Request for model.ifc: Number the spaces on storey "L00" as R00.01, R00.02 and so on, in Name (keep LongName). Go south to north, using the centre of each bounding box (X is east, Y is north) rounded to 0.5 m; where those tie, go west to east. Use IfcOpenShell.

First a look at what the model holds.

```python
import ifcopenshell
import ifcopenshell.util.element
import ifcopenshell.util.placement

model = ifcopenshell.open("model.ifc")
print(model.schema)
storey = next(s for s in model.by_type("IfcBuildingStorey") if s.Name == "L00")
spaces = [e for e in ifcopenshell.util.element.get_decomposition(storey) if e.is_a("IfcSpace")]
for e in sorted(spaces, key=lambda e: e.id()):
    origin = ifcopenshell.util.placement.get_local_placement(e.ObjectPlacement)[:3, 3]
    print(e.id(), e.Name, e.LongName, origin.round(2) + 0.0, sep=" | ")
```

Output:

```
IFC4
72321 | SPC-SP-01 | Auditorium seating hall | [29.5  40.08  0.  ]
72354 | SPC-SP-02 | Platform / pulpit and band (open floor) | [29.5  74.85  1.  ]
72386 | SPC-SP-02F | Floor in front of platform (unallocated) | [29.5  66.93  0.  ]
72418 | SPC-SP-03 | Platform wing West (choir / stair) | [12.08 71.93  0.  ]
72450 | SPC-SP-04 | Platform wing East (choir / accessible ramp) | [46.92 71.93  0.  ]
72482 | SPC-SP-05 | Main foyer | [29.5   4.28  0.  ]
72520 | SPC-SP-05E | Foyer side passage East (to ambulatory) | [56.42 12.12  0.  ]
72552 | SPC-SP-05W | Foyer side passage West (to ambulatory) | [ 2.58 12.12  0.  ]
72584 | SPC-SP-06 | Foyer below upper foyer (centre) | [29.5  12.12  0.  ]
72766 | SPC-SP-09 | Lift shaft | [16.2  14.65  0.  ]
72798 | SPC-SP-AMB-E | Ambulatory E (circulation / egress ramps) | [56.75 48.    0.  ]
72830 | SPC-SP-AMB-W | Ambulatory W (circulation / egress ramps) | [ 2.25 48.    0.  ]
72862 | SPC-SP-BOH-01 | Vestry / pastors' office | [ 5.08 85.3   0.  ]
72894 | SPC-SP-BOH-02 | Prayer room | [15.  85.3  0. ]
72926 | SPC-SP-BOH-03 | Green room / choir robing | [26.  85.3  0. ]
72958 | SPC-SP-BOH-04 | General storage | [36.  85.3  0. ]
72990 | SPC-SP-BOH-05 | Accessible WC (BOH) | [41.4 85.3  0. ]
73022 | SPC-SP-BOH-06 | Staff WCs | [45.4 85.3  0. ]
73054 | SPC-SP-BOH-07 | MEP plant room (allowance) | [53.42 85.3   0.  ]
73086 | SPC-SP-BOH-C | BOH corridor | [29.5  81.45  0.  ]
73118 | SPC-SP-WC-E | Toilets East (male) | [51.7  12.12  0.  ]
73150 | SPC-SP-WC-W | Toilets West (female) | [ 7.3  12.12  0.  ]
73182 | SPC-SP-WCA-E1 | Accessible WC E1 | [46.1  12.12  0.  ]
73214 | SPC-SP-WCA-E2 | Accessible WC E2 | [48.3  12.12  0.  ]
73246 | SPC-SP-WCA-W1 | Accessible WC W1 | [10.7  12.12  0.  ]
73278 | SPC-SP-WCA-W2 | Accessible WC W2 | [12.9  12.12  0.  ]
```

```python
import ifcopenshell
import ifcopenshell.geom
import ifcopenshell.util.element
import ifcopenshell.util.shape

model = ifcopenshell.open("model.ifc")
settings = ifcopenshell.geom.settings()
settings.set("use-world-coords", True)


def centre(element):
    shape = ifcopenshell.geom.create_shape(settings, element)
    return ifcopenshell.util.shape.get_bbox_centroid(shape.geometry)


storey = next(s for s in model.by_type("IfcBuildingStorey") if s.Name == "L00")
spaces = [e for e in ifcopenshell.util.element.get_decomposition(storey) if e.is_a("IfcSpace")]

# Insertion points can sit at a corner or the storey origin, so sort by the geometry (in metres).
centres = {e: centre(e) for e in spaces}
spaces.sort(key=lambda e: (round(centres[e][1] / 0.5), centres[e][0]))

for i, e in enumerate(spaces, start=1):
    number = f"R00.{i:02d}"
    e.Name = number
    print(e.id(), number)

model.write("model-out.ifc")
```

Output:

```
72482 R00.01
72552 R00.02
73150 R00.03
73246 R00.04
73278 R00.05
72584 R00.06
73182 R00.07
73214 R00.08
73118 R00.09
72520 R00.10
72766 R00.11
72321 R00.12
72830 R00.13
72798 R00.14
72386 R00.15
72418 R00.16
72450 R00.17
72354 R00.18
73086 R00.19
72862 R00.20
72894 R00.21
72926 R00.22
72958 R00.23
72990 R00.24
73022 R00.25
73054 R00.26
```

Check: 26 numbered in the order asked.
